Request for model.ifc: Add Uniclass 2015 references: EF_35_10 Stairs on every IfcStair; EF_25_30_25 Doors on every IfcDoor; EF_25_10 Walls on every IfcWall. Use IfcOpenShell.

First a look at what the model holds.

```python
import ifcopenshell

model = ifcopenshell.open("model.ifc")
print(model.schema)
print("classifications:", [c.Name for c in model.by_type("IfcClassification")])
for ifc_class in ("IfcDoor", "IfcRoof", "IfcStair", "IfcWall", "IfcWindow"):
    print(ifc_class, len(model.by_type(ifc_class)))
```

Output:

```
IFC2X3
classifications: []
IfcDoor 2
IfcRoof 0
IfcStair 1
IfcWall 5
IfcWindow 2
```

```python
import ifcopenshell
import ifcopenshell.api.classification

model = ifcopenshell.open("model.ifc")

# IFC2X3 requires Source and Edition and has no link from the project to the system.
system = model.create_entity("IfcClassification", Source="NBS", Edition="2015", Name="Uniclass 2015")

codes = {
    "IfcStair": ("EF_35_10", "Stairs"),
    "IfcDoor": ("EF_25_30_25", "Doors"),
    "IfcWall": ("EF_25_10", "Walls"),
}
for ifc_class, (code, name) in codes.items():
    products = model.by_type(ifc_class)
    ifcopenshell.api.classification.add_reference(
        model, products=products, classification=system, identification=code, name=name
    )
    print(code, len(products))

model.write("model-out.ifc")
```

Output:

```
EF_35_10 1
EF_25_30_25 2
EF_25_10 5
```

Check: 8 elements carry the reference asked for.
